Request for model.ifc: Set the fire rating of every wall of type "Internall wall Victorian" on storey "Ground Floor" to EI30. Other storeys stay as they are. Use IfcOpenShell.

First a look at what the model holds.

```python
import ifcopenshell
import ifcopenshell.util.element

model = ifcopenshell.open("model.ifc")
print(model.schema)
storey = next(s for s in model.by_type("IfcBuildingStorey") if s.Name == "Ground Floor")
walls = [e for e in ifcopenshell.util.element.get_decomposition(storey) if e.is_a("IfcWall")]
seen = {}
for e in walls:
    element_type = ifcopenshell.util.element.get_type(e)
    key = (element_type.Name if element_type != e and element_type else None, ifcopenshell.util.element.get_pset(e, "Pset_WallCommon", "FireRating"))
    seen[key] = seen.get(key, 0) + 1
for (name, value), count in sorted(seen.items(), key=str):
    print(count, "x", name, "|", value)
```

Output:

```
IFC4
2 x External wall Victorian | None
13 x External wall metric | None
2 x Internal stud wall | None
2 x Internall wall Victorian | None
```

```python
import ifcopenshell
import ifcopenshell.api.pset
import ifcopenshell.util.element

model = ifcopenshell.open("model.ifc")

storey = next(s for s in model.by_type("IfcBuildingStorey") if s.Name == "Ground Floor")
walls = [e for e in ifcopenshell.util.element.get_decomposition(storey) if e.is_a("IfcWall")]

count = 0
for e in walls:
    element_type = ifcopenshell.util.element.get_type(e)
    if element_type in (None, e) or element_type.Name != "Internall wall Victorian":
        continue
    # add_pset returns the element's existing set when there is one.
    pset = ifcopenshell.api.pset.add_pset(model, product=e, name="Pset_WallCommon")
    ifcopenshell.api.pset.edit_pset(model, pset=pset, properties={"FireRating": "EI30"})
    count += 1

print(count, "walls updated")

model.write("model_edited.ifc")
```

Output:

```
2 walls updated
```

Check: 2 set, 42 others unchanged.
